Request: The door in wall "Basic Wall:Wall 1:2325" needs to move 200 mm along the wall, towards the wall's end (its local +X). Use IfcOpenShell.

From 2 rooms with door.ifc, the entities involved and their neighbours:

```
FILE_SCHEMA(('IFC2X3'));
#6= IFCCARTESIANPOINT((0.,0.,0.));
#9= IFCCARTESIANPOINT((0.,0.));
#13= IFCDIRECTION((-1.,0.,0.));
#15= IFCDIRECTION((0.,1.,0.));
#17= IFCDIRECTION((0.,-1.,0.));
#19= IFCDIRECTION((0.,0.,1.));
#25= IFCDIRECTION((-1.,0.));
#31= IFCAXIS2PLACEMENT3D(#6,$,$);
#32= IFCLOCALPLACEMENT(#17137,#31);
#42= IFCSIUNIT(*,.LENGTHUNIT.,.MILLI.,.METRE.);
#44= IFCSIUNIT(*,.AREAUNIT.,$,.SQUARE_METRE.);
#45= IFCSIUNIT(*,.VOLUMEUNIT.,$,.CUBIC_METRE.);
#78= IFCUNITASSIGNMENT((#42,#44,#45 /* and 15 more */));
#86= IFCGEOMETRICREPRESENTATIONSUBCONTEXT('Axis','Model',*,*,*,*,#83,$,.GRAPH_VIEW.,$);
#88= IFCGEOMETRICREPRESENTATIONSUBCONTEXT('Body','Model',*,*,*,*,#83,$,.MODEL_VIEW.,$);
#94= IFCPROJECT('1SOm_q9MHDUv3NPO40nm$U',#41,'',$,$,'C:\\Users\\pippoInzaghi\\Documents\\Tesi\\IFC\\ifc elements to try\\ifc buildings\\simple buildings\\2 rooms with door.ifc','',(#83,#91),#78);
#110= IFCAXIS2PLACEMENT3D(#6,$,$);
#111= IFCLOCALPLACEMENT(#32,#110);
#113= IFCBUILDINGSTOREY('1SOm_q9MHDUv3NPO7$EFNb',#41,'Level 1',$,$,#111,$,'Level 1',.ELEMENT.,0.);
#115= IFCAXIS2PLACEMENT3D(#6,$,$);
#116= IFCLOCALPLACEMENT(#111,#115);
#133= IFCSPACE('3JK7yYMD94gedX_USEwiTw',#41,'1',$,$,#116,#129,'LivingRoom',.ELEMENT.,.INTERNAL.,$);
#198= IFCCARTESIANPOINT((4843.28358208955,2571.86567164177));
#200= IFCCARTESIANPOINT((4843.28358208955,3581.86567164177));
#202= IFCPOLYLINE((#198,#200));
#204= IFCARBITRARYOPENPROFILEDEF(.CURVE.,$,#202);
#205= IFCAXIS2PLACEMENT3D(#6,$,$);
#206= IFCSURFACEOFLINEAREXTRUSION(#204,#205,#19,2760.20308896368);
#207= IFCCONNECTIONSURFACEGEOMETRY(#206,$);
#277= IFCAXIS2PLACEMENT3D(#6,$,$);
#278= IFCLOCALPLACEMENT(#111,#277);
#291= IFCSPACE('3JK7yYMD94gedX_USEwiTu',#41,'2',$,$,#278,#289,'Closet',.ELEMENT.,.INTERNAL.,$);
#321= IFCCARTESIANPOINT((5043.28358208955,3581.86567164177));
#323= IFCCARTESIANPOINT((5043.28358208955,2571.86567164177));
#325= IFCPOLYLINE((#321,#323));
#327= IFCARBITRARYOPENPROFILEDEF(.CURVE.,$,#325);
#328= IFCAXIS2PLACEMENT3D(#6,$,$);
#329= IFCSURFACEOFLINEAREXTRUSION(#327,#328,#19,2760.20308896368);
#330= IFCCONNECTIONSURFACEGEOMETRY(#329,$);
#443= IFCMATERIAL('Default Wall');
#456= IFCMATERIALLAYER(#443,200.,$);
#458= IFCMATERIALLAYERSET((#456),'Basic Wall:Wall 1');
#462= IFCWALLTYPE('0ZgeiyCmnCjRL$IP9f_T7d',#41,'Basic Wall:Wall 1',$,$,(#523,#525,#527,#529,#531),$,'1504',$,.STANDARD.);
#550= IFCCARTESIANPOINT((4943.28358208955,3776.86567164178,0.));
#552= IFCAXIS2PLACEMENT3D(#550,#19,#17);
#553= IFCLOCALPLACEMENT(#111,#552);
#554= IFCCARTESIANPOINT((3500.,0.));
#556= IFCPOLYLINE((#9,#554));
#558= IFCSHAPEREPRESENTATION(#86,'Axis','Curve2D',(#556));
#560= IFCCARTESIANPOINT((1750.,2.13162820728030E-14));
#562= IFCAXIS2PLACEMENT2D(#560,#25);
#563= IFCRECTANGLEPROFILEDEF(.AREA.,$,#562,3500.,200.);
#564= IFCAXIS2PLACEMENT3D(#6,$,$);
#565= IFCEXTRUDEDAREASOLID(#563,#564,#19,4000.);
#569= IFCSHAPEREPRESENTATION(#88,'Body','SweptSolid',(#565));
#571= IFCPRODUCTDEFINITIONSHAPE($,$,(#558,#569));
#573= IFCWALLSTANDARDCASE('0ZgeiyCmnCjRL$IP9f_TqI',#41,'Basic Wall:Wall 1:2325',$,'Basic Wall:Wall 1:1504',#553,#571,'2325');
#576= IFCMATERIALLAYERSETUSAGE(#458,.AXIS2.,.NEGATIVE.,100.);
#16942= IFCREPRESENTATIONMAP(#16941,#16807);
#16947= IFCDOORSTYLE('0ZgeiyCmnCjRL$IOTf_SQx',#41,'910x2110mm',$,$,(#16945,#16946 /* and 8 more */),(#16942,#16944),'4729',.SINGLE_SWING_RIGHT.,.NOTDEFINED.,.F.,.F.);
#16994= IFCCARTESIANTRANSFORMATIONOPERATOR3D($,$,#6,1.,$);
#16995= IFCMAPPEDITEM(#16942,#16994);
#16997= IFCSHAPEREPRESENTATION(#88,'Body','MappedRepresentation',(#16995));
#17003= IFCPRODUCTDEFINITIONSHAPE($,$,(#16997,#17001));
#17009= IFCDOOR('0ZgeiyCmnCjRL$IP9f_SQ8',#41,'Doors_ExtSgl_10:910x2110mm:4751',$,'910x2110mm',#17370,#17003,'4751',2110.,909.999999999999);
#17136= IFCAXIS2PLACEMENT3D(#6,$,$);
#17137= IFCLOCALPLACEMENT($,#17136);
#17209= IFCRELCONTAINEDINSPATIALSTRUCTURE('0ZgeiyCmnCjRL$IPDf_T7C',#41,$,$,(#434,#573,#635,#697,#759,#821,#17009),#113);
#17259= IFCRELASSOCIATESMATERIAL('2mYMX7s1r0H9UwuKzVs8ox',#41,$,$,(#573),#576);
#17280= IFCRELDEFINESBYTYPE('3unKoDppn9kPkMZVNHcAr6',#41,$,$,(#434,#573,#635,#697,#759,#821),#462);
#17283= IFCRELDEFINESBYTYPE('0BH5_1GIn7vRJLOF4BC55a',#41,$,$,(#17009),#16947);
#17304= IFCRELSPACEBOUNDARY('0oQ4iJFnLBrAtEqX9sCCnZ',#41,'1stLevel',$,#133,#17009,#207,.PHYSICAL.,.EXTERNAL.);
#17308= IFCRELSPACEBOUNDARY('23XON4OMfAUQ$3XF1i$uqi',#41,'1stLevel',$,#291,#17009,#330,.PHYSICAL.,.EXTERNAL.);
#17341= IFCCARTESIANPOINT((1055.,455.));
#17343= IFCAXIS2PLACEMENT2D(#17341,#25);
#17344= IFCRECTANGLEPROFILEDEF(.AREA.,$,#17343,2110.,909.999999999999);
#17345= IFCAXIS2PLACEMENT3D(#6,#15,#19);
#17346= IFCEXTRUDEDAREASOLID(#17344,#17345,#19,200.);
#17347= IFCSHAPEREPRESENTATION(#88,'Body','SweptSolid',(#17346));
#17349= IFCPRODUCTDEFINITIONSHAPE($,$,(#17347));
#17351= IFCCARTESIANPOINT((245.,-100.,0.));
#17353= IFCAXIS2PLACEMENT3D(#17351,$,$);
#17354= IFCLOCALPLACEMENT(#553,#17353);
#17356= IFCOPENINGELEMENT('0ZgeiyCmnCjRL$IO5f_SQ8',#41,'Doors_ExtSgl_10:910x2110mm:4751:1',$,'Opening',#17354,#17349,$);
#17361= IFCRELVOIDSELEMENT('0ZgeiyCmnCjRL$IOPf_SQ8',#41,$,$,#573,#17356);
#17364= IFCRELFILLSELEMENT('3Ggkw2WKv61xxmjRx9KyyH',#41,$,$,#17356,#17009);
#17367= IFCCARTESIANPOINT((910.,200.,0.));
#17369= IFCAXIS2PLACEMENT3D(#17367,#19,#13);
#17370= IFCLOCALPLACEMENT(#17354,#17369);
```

```python
import numpy as np
import ifcopenshell
import ifcopenshell.api.geometry
import ifcopenshell.util.placement
import ifcopenshell.util.unit

model = ifcopenshell.open("2 rooms with door.ifc")
unit_scale = ifcopenshell.util.unit.calculate_unit_scale(model)

door = model.by_id(17009)
opening = door.FillsVoids[0].RelatingOpeningElement
wall = opening.VoidsElements[0].RelatingBuildingElement

wall_matrix = ifcopenshell.util.placement.get_local_placement(wall.ObjectPlacement)
shift = wall_matrix[:3, 0] * 0.2 / unit_scale
before = ifcopenshell.util.placement.get_local_placement(door.ObjectPlacement)[:3, 3].copy()

# The door is placed relative to its opening, so it follows when the opening moves.
matrix = ifcopenshell.util.placement.get_local_placement(opening.ObjectPlacement)
matrix[:3, 3] += shift
ifcopenshell.api.geometry.edit_object_placement(
    model, product=opening, matrix=matrix, is_si=False, should_transform_children=True
)

# Space boundary surfaces are stored in each space's coordinates; move them too.
for rel in door.ProvidesBoundaries:
    if not rel.ConnectionGeometry:
        continue
    surface = rel.ConnectionGeometry.SurfaceOnRelatingElement
    space_matrix = ifcopenshell.util.placement.get_local_placement(rel.RelatingSpace.ObjectPlacement)
    point = np.array(surface.Position.Location.Coordinates) + space_matrix[:3, :3].T @ shift
    surface.Position = model.createIfcAxis2Placement3D(
        model.createIfcCartesianPoint(point.tolist()), surface.Position.Axis, surface.Position.RefDirection
    )

after = ifcopenshell.util.placement.get_local_placement(door.ObjectPlacement)[:3, 3]
print("door moved by", (after - before).round(3) + 0.0)

model.write("2 rooms with door_v2.ifc")
```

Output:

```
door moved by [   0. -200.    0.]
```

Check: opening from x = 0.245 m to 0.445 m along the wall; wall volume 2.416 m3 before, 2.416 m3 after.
